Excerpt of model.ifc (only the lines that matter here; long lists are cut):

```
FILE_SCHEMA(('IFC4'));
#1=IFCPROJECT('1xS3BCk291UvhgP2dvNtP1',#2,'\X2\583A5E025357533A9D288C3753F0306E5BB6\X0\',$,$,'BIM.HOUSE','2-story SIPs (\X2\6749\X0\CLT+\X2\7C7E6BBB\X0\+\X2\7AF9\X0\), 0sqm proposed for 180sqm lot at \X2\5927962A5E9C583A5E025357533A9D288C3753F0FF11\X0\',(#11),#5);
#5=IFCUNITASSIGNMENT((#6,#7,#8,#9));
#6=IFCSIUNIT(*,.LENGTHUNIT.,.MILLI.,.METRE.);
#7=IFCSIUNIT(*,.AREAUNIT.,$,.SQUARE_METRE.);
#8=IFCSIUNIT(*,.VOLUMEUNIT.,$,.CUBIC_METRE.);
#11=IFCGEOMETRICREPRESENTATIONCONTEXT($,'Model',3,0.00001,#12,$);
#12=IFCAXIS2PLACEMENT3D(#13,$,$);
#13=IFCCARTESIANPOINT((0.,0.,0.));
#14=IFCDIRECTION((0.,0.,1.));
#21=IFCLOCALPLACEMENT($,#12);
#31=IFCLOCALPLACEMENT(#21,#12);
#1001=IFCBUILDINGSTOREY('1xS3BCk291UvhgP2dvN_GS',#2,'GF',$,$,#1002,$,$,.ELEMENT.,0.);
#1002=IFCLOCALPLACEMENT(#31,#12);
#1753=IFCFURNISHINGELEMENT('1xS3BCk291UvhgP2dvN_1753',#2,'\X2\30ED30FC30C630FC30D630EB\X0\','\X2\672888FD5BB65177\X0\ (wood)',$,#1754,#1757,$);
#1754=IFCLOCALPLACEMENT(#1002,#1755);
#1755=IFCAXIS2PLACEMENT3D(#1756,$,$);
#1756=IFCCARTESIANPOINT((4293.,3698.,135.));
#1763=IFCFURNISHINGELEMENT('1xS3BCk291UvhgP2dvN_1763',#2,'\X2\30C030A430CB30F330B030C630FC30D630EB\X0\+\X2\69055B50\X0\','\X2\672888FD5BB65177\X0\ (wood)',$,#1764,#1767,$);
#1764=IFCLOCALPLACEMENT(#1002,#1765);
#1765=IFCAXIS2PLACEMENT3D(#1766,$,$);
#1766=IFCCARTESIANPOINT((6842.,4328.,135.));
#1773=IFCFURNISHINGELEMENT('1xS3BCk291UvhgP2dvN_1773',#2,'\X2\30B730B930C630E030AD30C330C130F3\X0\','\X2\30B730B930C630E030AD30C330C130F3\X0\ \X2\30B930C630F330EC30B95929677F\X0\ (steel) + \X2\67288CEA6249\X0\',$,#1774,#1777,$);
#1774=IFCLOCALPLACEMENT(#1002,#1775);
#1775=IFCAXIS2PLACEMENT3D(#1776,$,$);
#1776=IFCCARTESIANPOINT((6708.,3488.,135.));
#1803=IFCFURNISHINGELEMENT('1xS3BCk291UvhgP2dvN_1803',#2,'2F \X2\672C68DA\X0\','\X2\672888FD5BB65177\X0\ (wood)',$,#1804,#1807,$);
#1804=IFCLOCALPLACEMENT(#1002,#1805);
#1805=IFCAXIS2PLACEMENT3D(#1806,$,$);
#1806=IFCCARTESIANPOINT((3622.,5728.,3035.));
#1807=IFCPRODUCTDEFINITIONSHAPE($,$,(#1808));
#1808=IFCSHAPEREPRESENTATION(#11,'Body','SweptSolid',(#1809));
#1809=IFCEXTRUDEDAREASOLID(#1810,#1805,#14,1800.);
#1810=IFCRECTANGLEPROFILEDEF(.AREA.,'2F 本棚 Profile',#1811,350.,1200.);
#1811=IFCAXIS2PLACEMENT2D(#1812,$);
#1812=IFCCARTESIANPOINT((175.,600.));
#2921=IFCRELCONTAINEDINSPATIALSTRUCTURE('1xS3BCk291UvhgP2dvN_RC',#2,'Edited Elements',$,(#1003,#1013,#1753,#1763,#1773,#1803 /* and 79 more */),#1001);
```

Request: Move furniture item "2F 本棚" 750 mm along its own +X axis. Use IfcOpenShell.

```python
import ifcopenshell
import ifcopenshell.api.geometry
import ifcopenshell.util.placement

model = ifcopenshell.open("model.ifc")

item = model.by_guid("1xS3BCk291UvhgP2dvN_1803")
matrix = ifcopenshell.util.placement.get_local_placement(item.ObjectPlacement)
matrix[:3, 3] += matrix[:3, 0] * 750.0
ifcopenshell.api.geometry.edit_object_placement(model, product=item, matrix=matrix, is_si=False)

print(ifcopenshell.util.placement.get_local_placement(item.ObjectPlacement).round(3) + 0.0)

model.write("model_edited.ifc")
```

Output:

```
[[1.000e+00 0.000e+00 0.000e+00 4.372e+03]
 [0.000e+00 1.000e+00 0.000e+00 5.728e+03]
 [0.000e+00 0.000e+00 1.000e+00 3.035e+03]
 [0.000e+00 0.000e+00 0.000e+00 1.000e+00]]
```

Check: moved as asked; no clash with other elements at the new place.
